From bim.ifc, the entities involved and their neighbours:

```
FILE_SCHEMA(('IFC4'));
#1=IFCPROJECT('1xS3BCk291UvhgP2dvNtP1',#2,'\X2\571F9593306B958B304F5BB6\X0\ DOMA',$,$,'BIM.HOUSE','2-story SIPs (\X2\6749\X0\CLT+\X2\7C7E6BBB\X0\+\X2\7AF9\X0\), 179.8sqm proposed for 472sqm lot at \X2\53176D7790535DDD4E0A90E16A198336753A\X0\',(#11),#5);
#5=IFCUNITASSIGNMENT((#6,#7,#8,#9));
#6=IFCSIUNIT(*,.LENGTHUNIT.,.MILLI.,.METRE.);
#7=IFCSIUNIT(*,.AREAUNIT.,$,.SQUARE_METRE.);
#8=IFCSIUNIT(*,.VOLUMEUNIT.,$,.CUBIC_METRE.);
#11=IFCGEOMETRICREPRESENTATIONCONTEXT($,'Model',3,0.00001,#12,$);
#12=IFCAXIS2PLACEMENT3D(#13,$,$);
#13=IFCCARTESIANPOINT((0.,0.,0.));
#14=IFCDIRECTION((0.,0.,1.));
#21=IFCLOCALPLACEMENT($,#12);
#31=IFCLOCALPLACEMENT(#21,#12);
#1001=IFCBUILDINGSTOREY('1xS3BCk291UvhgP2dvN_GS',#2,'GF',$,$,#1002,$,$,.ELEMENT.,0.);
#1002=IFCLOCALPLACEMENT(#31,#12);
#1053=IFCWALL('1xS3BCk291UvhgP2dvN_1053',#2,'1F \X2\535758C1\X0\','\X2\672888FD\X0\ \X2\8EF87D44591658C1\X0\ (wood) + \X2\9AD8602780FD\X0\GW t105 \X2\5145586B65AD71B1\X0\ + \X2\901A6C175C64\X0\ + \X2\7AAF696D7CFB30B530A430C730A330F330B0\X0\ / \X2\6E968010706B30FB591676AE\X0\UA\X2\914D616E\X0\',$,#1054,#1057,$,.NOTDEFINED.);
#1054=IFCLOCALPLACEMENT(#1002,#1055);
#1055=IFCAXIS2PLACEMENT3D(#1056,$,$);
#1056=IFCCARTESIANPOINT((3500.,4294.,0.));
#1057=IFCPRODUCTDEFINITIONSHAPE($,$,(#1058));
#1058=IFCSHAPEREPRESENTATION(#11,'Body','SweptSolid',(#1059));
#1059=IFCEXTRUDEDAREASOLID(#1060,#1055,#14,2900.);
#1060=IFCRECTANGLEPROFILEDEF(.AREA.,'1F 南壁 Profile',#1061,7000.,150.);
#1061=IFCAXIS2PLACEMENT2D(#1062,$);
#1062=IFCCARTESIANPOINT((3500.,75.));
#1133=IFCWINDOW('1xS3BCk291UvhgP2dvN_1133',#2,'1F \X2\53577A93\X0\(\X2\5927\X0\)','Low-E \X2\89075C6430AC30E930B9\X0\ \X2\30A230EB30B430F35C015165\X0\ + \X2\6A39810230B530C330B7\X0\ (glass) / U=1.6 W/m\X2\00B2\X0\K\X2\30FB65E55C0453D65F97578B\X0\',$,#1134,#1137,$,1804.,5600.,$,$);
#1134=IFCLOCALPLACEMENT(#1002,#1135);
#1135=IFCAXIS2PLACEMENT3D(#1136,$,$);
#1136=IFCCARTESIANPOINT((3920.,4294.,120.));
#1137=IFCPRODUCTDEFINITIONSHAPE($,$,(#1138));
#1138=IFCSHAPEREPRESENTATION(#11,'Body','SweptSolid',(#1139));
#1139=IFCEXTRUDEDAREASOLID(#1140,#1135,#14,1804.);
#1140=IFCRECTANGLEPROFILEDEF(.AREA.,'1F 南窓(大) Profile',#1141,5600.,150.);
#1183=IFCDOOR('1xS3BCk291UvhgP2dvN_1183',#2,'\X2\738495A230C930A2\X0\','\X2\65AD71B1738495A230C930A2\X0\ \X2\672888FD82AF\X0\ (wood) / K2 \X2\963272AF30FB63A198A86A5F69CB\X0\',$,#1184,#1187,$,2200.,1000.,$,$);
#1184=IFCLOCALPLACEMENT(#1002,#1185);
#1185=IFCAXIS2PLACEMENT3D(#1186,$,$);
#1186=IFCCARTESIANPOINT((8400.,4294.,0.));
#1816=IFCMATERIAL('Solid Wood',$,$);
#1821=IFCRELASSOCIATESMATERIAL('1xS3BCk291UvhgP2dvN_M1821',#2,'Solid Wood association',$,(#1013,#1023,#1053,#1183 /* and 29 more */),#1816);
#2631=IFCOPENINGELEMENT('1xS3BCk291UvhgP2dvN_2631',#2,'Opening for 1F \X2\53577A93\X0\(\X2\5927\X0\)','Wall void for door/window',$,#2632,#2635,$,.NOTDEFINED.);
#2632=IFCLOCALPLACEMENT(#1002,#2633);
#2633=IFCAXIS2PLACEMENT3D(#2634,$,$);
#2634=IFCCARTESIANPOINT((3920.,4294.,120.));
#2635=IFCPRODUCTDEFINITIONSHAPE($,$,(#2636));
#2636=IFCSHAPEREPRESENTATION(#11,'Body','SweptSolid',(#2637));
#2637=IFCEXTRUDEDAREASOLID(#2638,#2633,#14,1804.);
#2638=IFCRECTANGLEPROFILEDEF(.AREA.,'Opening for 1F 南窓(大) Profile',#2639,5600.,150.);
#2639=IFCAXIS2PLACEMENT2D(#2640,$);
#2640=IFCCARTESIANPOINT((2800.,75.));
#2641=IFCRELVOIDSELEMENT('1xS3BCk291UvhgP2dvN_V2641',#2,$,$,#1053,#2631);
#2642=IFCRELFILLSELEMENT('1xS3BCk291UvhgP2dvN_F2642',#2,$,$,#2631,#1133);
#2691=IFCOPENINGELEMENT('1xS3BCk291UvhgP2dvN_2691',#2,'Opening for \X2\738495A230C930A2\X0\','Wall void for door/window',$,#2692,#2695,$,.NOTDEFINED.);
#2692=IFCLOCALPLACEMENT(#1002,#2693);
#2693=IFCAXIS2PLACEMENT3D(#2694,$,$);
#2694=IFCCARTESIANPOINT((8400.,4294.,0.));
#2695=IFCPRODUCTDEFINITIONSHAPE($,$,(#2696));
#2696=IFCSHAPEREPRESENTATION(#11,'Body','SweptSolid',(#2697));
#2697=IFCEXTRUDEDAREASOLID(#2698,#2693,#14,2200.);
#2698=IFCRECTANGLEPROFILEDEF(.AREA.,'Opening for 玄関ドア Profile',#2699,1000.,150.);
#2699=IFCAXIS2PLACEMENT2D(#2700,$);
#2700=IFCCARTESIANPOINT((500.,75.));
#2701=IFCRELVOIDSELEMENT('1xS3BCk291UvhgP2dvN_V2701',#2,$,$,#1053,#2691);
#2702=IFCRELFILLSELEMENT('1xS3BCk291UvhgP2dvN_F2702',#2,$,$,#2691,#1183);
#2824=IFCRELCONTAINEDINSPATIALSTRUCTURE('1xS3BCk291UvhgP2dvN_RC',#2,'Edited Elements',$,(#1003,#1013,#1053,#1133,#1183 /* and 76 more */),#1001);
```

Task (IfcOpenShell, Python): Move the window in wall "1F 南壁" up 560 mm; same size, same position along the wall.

```python
import numpy as np
import ifcopenshell
import ifcopenshell.api.geometry
import ifcopenshell.util.placement
import ifcopenshell.util.unit

model = ifcopenshell.open("bim.ifc")
unit_scale = ifcopenshell.util.unit.calculate_unit_scale(model)

window = model.by_guid("1xS3BCk291UvhgP2dvN_1133")
opening = window.FillsVoids[0].RelatingOpeningElement
dz = 560.0

shift = np.array([0.0, 0.0, dz])
# The window is not placed relative to its opening, so move both.
for product in (opening, window):
    matrix = ifcopenshell.util.placement.get_local_placement(product.ObjectPlacement)
    matrix[:3, 3] += shift
    ifcopenshell.api.geometry.edit_object_placement(model, product=product, matrix=matrix, is_si=False)

print(f"moved by {dz * unit_scale:+.3f} m")

model.write("bim-out.ifc")
```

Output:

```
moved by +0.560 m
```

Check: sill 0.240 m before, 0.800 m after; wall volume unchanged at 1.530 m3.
